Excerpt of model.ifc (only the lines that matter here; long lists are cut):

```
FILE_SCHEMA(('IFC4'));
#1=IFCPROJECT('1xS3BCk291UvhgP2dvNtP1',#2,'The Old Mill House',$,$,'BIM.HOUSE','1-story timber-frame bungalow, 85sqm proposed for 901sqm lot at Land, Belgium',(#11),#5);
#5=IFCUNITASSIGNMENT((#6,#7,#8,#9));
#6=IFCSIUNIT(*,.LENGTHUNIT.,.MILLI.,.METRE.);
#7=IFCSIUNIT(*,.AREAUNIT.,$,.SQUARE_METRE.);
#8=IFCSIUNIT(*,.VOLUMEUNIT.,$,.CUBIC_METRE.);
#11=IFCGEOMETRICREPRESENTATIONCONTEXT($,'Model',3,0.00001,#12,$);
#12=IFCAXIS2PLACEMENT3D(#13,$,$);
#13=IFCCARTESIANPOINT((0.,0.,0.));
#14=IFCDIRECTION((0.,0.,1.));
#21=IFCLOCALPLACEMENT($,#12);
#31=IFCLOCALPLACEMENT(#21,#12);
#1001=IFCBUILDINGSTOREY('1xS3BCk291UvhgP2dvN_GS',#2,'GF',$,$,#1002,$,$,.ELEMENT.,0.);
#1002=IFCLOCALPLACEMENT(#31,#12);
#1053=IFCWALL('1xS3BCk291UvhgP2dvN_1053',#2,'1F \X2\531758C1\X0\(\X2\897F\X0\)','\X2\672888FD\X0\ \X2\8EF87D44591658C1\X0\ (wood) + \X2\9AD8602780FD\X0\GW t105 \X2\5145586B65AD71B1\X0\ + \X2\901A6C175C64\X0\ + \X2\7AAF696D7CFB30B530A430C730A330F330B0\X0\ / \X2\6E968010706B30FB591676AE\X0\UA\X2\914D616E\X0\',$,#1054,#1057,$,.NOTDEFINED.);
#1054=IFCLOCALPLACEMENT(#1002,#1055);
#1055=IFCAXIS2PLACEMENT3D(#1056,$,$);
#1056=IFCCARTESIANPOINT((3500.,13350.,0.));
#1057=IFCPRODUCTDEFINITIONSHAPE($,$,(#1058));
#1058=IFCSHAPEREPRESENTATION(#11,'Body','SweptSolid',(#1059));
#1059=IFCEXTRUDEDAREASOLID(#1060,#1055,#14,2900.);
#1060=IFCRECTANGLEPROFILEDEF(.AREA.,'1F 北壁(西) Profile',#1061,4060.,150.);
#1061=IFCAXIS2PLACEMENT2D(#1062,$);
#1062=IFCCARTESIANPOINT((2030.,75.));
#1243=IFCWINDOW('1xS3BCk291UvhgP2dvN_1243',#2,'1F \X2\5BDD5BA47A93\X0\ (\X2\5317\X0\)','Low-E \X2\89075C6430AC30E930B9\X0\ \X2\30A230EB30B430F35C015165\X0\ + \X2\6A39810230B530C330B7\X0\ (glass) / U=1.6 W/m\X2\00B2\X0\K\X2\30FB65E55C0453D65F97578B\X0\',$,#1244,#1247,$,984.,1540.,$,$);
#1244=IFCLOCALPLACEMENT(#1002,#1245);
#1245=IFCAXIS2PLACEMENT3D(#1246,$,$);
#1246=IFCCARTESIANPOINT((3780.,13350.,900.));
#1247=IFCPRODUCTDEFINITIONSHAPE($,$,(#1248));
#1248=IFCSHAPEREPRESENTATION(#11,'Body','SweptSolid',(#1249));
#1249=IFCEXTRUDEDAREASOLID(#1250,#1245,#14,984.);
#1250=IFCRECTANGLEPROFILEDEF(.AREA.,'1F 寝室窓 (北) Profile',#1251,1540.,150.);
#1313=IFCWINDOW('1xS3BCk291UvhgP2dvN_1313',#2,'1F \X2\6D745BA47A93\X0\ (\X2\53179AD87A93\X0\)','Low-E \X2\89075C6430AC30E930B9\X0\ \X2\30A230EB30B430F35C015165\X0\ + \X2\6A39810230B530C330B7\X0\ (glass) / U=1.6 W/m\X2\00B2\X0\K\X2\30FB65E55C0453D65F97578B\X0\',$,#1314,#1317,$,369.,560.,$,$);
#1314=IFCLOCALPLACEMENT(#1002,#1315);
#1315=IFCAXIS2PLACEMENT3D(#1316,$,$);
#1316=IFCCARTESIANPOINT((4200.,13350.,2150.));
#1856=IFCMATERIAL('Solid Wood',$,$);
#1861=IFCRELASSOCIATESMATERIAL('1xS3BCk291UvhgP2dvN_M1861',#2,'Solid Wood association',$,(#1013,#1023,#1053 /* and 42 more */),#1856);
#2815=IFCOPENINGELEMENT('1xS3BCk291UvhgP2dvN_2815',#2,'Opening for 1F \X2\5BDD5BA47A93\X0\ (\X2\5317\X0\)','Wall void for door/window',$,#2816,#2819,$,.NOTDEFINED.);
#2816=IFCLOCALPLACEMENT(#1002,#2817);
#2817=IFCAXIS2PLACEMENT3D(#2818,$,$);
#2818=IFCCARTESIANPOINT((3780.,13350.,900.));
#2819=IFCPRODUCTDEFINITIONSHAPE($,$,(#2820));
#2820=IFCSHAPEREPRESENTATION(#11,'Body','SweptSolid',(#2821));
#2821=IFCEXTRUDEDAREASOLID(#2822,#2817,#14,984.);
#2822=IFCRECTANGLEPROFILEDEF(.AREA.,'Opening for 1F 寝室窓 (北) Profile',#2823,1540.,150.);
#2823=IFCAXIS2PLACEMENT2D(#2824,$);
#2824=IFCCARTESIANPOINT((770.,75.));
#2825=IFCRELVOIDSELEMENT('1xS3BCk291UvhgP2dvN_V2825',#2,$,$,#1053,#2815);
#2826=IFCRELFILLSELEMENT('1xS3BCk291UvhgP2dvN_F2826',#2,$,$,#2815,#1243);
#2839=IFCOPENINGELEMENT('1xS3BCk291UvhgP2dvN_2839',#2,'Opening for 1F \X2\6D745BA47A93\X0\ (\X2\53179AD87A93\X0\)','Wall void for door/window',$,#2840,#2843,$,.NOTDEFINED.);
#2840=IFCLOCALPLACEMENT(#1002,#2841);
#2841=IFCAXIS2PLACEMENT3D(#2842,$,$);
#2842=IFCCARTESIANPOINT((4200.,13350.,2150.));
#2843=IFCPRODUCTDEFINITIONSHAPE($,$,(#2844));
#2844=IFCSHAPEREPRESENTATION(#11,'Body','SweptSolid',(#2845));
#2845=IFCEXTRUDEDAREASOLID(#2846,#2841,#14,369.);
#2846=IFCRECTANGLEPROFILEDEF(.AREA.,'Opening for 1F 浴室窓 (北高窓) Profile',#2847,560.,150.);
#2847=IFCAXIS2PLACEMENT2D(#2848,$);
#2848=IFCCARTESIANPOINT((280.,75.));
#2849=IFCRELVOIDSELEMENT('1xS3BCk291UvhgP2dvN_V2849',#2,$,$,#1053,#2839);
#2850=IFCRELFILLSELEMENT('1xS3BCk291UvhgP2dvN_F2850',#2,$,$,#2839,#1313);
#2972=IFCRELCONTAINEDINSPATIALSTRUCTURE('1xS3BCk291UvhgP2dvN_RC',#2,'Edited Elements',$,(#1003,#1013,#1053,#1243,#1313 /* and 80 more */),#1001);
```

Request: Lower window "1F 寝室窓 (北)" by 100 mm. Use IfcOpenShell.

```python
import numpy as np
import ifcopenshell
import ifcopenshell.api.geometry
import ifcopenshell.util.placement
import ifcopenshell.util.unit

model = ifcopenshell.open("model.ifc")
unit_scale = ifcopenshell.util.unit.calculate_unit_scale(model)

window = model.by_guid("1xS3BCk291UvhgP2dvN_1243")
opening = window.FillsVoids[0].RelatingOpeningElement
dz = -100.0

shift = np.array([0.0, 0.0, dz])
# The window is not placed relative to its opening, so move both.
for product in (opening, window):
    matrix = ifcopenshell.util.placement.get_local_placement(product.ObjectPlacement)
    matrix[:3, 3] += shift
    ifcopenshell.api.geometry.edit_object_placement(model, product=product, matrix=matrix, is_si=False)

print(f"moved by {dz * unit_scale:+.3f} m")

model.write("model_v2.ifc")
```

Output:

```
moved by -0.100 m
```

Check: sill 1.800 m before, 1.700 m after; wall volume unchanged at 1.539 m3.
